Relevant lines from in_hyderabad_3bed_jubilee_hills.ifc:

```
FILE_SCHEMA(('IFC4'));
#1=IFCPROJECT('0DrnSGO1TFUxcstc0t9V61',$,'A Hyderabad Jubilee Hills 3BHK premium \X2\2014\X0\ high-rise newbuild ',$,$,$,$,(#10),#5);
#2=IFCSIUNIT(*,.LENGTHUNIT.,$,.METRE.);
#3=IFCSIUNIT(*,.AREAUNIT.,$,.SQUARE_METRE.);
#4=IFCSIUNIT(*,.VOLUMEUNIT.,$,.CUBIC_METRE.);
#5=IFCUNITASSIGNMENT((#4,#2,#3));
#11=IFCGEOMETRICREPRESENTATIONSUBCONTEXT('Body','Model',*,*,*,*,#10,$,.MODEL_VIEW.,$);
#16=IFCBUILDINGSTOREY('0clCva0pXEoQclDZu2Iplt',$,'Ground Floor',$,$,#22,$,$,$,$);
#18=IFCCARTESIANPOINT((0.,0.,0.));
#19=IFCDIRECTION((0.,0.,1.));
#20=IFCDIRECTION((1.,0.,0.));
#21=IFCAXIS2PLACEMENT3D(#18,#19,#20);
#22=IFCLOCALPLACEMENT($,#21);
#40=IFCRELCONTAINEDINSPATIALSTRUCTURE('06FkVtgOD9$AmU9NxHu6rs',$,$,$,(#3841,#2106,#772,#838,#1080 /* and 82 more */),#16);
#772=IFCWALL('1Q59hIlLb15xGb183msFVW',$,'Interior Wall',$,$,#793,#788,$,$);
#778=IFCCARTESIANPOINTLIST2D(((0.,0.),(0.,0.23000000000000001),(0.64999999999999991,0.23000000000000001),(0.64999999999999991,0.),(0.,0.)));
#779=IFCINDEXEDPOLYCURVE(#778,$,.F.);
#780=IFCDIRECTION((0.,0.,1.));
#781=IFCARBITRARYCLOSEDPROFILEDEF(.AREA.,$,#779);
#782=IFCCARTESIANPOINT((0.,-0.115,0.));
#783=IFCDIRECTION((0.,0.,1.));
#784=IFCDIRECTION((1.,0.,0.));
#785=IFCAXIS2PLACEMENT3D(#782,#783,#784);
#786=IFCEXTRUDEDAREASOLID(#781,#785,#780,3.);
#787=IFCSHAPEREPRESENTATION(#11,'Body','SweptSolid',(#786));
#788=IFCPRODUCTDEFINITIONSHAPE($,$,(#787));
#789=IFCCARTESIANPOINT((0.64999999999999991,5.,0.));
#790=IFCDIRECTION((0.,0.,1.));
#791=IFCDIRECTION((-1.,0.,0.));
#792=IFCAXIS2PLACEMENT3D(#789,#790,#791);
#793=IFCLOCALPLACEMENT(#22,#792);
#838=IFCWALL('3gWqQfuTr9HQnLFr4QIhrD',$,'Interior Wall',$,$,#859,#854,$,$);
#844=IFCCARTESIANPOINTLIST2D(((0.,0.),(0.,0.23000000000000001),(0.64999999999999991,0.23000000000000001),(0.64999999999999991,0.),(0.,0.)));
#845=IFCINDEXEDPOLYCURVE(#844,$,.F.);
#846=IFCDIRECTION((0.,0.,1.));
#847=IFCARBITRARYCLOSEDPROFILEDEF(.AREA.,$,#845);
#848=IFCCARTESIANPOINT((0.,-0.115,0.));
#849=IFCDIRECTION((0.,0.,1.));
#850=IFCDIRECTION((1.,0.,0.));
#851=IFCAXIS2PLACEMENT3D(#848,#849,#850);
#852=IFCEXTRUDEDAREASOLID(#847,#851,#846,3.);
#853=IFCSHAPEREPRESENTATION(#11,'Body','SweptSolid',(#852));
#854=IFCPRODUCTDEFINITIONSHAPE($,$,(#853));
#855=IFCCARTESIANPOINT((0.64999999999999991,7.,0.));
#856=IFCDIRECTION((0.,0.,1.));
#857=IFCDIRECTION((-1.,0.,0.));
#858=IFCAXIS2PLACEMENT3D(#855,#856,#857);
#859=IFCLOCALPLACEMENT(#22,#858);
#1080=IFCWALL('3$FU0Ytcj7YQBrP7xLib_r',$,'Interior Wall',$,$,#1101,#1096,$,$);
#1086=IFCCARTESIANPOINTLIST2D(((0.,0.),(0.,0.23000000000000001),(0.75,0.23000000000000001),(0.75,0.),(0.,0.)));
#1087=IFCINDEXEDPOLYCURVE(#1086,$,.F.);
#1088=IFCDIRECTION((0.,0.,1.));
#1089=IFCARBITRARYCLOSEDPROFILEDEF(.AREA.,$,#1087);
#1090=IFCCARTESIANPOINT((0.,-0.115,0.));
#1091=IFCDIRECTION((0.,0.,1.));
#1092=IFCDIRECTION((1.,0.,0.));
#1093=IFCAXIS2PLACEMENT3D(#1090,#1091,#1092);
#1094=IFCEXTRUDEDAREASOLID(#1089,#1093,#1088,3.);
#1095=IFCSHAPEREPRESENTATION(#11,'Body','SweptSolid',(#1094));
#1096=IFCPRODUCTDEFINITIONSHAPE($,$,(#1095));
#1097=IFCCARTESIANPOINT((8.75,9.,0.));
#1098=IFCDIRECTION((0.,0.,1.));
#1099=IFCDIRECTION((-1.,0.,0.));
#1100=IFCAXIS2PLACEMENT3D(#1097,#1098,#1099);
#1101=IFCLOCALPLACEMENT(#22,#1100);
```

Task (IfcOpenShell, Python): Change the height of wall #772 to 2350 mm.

```python
import ifcopenshell
import ifcopenshell.geom
import ifcopenshell.util.representation
import ifcopenshell.util.shape
import ifcopenshell.util.unit

model = ifcopenshell.open("in_hyderabad_3bed_jubilee_hills.ifc")
unit_scale = ifcopenshell.util.unit.calculate_unit_scale(model)
settings = ifcopenshell.geom.settings()


def volume(element):
    """Net volume in cubic metres, openings subtracted."""
    shape = ifcopenshell.geom.create_shape(settings, element)
    return ifcopenshell.util.shape.get_volume(shape.geometry)


wall = model.by_guid("1Q59hIlLb15xGb183msFVW")
before = volume(wall)

body = ifcopenshell.util.representation.get_representation(wall, "Model", "Body")
solid = body.Items[0]
old_height = solid.Depth
solid.Depth = 2.35 / unit_scale
after = volume(wall)

print(f"height {old_height:g} -> {solid.Depth:g}, volume {before:.3f} -> {after:.3f} m3")

model.write("in_hyderabad_3bed_jubilee_hills_v2.ifc")
```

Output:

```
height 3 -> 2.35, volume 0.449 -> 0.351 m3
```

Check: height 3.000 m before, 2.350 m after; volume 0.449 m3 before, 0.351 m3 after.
